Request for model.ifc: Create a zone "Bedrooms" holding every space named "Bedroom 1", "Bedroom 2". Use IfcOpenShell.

First a look at what the model holds.

```python
import ifcopenshell

model = ifcopenshell.open("model.ifc")
print(model.schema)
seen = {}
for space in model.by_type("IfcSpace"):
    seen[space.LongName] = seen.get(space.LongName, 0) + 1
for name, count in sorted(seen.items(), key=str):
    print(count, "x", name)
print("zones:", [z.Name for z in model.by_type("IfcZone")][:20])
```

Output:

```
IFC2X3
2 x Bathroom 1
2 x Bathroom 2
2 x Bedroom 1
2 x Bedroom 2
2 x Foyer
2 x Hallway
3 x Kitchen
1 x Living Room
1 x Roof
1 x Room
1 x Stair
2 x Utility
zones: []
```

```python
import ifcopenshell
import ifcopenshell.api.group
import ifcopenshell.api.root

model = ifcopenshell.open("model.ifc")

names = {"Bedroom 1", "Bedroom 2"}
spaces = [s for s in model.by_type("IfcSpace") if s.LongName in names]

zone = ifcopenshell.api.root.create_entity(model, ifc_class="IfcZone", name="Bedrooms")
ifcopenshell.api.group.assign_group(model, products=spaces, group=zone)
print(len(spaces), "spaces in", zone.Name)

model.write("model_rev.ifc")
```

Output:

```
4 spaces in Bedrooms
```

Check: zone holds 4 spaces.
